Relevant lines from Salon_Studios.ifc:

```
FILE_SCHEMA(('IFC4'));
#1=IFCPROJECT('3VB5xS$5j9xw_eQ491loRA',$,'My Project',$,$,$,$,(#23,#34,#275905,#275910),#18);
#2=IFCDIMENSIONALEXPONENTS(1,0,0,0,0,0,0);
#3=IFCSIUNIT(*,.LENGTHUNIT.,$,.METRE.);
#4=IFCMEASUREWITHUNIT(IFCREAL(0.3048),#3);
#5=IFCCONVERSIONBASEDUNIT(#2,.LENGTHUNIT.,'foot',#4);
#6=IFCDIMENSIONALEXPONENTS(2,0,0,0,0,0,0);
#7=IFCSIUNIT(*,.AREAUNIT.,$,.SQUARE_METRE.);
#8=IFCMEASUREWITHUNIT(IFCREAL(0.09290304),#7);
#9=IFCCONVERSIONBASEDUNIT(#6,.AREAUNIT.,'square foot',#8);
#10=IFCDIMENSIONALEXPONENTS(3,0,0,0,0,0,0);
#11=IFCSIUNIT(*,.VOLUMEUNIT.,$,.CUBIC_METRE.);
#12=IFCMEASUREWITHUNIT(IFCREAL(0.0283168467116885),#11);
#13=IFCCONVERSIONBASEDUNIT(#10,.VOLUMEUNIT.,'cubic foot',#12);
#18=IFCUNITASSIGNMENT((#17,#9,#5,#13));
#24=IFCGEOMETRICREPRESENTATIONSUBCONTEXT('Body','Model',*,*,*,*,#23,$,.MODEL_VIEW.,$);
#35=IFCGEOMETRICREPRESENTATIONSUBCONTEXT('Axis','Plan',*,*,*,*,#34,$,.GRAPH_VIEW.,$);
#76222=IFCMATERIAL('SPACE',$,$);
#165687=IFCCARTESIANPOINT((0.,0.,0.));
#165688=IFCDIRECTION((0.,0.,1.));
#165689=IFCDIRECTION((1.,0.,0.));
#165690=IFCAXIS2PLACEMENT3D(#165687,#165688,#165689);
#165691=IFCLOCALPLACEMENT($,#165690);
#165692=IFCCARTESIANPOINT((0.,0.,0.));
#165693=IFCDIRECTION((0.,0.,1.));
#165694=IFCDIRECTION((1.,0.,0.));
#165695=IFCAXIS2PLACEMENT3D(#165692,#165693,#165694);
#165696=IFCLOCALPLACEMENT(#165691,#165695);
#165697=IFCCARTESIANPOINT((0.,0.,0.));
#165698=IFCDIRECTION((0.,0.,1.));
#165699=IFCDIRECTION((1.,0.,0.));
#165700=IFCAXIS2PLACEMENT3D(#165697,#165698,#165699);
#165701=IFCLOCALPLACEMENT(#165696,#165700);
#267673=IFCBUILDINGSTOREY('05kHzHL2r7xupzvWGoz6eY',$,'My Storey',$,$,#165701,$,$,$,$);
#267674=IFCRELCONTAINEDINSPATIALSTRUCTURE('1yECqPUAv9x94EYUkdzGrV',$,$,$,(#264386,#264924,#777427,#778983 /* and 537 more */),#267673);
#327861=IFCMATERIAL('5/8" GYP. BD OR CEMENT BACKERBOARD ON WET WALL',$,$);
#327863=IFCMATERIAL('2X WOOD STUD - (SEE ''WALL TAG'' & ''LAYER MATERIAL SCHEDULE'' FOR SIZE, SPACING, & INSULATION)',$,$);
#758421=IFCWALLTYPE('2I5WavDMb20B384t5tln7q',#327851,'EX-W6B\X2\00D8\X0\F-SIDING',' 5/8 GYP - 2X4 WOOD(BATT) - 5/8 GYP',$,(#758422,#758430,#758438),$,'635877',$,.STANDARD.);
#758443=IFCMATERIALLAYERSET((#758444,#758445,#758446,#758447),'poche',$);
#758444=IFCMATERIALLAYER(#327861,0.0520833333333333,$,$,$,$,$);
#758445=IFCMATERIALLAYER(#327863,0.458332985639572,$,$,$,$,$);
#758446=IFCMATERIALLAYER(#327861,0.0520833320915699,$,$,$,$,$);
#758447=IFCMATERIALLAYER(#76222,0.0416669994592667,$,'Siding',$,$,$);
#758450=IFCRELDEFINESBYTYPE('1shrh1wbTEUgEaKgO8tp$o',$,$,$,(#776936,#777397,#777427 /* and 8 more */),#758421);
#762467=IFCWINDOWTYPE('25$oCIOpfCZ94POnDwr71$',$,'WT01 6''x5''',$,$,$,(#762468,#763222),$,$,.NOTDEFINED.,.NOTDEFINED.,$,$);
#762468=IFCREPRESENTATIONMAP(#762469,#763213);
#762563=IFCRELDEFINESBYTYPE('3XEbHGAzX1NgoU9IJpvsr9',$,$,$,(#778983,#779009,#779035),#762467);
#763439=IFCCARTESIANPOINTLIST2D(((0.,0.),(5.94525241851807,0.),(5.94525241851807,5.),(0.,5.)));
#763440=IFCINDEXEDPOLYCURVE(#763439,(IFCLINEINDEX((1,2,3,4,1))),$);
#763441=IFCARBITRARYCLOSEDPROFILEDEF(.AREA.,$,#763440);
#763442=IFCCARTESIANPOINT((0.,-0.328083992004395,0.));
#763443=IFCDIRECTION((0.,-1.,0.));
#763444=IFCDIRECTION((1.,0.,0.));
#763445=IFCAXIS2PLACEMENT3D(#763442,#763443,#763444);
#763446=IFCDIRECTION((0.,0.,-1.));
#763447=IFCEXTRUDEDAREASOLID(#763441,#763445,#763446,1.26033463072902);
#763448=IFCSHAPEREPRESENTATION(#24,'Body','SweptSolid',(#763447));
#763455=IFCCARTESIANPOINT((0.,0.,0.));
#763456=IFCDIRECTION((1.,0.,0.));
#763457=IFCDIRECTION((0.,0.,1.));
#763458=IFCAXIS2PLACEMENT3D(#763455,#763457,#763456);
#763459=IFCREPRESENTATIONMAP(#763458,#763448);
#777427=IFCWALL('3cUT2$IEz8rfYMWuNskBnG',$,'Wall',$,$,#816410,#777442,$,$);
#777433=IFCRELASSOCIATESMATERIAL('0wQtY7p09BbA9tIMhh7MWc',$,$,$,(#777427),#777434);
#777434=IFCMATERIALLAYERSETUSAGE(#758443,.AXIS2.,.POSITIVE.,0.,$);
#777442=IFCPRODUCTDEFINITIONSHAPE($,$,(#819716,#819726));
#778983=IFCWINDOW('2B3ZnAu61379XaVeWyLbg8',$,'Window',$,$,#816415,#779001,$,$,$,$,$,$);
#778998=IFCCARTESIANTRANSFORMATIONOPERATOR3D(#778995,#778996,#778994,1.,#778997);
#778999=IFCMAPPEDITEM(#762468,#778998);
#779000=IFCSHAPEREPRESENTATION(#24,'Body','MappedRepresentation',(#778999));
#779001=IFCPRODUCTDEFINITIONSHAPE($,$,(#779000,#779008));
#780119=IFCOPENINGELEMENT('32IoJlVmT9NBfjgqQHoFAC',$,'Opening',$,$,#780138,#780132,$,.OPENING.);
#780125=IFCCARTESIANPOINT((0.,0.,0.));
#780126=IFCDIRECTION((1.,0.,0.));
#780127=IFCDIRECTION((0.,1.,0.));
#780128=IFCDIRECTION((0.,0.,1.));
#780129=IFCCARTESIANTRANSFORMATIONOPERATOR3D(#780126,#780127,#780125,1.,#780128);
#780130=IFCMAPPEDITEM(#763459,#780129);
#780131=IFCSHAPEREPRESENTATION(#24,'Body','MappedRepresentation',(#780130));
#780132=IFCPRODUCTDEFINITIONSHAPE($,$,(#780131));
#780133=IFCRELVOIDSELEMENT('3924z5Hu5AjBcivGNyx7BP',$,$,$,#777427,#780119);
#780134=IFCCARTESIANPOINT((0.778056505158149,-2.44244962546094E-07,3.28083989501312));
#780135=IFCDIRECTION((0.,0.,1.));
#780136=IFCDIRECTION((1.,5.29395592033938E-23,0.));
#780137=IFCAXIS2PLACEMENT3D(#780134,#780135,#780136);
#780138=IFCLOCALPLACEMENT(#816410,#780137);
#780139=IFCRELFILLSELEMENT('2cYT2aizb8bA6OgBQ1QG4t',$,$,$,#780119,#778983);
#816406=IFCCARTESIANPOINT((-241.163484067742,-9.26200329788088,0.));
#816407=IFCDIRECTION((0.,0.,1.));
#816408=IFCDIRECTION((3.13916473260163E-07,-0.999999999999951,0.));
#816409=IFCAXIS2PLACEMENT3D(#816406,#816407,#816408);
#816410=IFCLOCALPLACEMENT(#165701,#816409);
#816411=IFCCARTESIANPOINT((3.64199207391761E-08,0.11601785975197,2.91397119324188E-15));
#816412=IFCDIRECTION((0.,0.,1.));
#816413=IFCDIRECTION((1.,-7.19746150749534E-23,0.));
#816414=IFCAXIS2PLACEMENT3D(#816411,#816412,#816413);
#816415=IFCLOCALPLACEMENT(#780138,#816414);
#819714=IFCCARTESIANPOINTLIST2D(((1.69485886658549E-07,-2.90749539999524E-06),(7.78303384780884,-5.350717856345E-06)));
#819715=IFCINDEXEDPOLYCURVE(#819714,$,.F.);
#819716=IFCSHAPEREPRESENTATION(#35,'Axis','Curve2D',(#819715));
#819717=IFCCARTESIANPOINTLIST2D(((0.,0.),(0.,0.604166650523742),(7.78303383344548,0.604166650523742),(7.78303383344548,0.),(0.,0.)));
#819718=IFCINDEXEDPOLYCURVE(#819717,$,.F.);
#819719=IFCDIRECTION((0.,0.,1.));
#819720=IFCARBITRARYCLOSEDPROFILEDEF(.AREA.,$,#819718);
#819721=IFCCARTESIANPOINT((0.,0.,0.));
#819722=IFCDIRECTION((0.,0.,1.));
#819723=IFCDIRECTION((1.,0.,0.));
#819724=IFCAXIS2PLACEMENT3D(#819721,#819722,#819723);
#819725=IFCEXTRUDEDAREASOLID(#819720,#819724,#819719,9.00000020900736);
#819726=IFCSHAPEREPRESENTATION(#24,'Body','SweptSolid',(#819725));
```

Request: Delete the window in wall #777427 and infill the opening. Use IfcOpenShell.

```python
import ifcopenshell
import ifcopenshell.api.feature
import ifcopenshell.api.root
import ifcopenshell.geom
import ifcopenshell.util.shape

model = ifcopenshell.open("Salon_Studios.ifc")
settings = ifcopenshell.geom.settings()


def volume(element):
    """Net volume in cubic metres, openings subtracted."""
    shape = ifcopenshell.geom.create_shape(settings, element)
    return ifcopenshell.util.shape.get_volume(shape.geometry)


window = model.by_guid("2B3ZnAu61379XaVeWyLbg8")
opening = window.FillsVoids[0].RelatingOpeningElement
wall = opening.VoidsElements[0].RelatingBuildingElement
before = volume(wall)

ifcopenshell.api.root.remove_product(model, product=window)
ifcopenshell.api.feature.remove_feature(model, feature=opening)

after = volume(wall)

print(f"wall volume {before:.3f} -> {after:.3f} m3")

model.write("Salon_Studios_edited.ifc")
```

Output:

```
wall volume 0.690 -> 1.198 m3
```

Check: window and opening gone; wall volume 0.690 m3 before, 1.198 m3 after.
